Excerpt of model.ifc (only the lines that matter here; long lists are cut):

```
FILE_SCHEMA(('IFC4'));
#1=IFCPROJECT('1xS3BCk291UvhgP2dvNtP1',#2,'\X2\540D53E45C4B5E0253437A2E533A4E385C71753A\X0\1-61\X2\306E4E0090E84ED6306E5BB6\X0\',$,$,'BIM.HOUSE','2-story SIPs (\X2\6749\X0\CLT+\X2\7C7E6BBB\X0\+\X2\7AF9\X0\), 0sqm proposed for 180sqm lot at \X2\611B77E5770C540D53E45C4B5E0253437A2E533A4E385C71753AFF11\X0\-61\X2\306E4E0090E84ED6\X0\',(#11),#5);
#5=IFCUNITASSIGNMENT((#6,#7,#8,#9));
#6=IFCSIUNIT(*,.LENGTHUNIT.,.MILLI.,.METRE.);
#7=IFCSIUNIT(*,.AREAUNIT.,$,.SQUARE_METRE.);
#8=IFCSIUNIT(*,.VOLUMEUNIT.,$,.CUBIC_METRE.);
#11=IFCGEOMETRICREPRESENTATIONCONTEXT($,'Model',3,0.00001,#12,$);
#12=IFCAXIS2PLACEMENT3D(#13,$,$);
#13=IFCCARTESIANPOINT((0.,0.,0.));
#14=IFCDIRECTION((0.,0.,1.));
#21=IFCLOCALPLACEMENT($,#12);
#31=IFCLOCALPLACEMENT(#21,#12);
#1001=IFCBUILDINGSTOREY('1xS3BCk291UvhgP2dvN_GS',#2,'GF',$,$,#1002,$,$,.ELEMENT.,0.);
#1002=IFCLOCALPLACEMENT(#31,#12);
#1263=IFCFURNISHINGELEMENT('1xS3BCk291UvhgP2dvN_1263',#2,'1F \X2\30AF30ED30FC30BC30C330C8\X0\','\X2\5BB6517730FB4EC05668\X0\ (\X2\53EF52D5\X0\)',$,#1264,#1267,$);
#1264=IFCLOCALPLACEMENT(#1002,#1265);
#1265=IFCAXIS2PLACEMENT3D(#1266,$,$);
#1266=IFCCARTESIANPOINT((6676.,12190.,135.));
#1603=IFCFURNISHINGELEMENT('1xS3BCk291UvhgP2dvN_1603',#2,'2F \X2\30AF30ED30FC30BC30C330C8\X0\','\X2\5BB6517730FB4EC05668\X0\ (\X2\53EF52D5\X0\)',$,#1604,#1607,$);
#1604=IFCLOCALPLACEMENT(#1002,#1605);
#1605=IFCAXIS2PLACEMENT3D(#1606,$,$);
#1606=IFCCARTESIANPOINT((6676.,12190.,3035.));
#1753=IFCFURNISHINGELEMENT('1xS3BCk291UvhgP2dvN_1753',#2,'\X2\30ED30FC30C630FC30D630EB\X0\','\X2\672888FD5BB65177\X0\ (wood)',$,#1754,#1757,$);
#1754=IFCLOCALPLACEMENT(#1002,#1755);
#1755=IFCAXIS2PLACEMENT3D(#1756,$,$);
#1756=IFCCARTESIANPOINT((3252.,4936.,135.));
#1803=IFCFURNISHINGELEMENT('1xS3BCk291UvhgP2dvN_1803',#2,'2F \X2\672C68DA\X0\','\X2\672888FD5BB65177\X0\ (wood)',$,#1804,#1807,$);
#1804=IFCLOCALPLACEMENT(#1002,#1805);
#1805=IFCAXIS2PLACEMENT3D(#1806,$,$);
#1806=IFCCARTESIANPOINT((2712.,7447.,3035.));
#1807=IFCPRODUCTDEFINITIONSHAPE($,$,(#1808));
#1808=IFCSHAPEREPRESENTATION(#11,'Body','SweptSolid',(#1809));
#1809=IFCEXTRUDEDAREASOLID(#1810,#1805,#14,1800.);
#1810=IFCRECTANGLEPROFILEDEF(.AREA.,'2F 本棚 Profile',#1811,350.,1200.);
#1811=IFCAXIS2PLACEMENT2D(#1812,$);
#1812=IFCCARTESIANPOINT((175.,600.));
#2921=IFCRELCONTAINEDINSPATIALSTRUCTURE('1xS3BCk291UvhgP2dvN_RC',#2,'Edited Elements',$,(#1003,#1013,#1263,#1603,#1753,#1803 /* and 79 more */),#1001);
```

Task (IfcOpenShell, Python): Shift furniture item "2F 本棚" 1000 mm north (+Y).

```python
import ifcopenshell
import ifcopenshell.api.geometry
import ifcopenshell.util.placement

model = ifcopenshell.open("model.ifc")

item = model.by_id(1803)
matrix = ifcopenshell.util.placement.get_local_placement(item.ObjectPlacement)
matrix[1, 3] += 1000.0
ifcopenshell.api.geometry.edit_object_placement(model, product=item, matrix=matrix, is_si=False)

print(ifcopenshell.util.placement.get_local_placement(item.ObjectPlacement).round(3) + 0.0)

model.write("model-out.ifc")
```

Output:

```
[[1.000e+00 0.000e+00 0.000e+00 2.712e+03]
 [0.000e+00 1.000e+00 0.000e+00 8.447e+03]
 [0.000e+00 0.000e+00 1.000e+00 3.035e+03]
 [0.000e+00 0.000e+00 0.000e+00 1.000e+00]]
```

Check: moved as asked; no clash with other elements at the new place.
